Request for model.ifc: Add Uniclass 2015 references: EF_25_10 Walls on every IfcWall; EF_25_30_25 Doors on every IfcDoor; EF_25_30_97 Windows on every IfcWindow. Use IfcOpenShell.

First a look at what the model holds.

```python
import ifcopenshell

model = ifcopenshell.open("model.ifc")
print(model.schema)
print("classifications:", [c.Name for c in model.by_type("IfcClassification")])
for ifc_class in ("IfcDoor", "IfcRoof", "IfcStair", "IfcWall", "IfcWindow"):
    print(ifc_class, len(model.by_type(ifc_class)))
```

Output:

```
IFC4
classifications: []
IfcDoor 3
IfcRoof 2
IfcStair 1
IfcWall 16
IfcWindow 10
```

```python
import ifcopenshell
import ifcopenshell.api.classification

model = ifcopenshell.open("model.ifc")

system = ifcopenshell.api.classification.add_classification(model, classification="Uniclass 2015")

codes = {
    "IfcWall": ("EF_25_10", "Walls"),
    "IfcDoor": ("EF_25_30_25", "Doors"),
    "IfcWindow": ("EF_25_30_97", "Windows"),
}
for ifc_class, (code, name) in codes.items():
    products = model.by_type(ifc_class)
    ifcopenshell.api.classification.add_reference(
        model, products=products, classification=system, identification=code, name=name
    )
    print(code, len(products))

model.write("model_v2.ifc")
```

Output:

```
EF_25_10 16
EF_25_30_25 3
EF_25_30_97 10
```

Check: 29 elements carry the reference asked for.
